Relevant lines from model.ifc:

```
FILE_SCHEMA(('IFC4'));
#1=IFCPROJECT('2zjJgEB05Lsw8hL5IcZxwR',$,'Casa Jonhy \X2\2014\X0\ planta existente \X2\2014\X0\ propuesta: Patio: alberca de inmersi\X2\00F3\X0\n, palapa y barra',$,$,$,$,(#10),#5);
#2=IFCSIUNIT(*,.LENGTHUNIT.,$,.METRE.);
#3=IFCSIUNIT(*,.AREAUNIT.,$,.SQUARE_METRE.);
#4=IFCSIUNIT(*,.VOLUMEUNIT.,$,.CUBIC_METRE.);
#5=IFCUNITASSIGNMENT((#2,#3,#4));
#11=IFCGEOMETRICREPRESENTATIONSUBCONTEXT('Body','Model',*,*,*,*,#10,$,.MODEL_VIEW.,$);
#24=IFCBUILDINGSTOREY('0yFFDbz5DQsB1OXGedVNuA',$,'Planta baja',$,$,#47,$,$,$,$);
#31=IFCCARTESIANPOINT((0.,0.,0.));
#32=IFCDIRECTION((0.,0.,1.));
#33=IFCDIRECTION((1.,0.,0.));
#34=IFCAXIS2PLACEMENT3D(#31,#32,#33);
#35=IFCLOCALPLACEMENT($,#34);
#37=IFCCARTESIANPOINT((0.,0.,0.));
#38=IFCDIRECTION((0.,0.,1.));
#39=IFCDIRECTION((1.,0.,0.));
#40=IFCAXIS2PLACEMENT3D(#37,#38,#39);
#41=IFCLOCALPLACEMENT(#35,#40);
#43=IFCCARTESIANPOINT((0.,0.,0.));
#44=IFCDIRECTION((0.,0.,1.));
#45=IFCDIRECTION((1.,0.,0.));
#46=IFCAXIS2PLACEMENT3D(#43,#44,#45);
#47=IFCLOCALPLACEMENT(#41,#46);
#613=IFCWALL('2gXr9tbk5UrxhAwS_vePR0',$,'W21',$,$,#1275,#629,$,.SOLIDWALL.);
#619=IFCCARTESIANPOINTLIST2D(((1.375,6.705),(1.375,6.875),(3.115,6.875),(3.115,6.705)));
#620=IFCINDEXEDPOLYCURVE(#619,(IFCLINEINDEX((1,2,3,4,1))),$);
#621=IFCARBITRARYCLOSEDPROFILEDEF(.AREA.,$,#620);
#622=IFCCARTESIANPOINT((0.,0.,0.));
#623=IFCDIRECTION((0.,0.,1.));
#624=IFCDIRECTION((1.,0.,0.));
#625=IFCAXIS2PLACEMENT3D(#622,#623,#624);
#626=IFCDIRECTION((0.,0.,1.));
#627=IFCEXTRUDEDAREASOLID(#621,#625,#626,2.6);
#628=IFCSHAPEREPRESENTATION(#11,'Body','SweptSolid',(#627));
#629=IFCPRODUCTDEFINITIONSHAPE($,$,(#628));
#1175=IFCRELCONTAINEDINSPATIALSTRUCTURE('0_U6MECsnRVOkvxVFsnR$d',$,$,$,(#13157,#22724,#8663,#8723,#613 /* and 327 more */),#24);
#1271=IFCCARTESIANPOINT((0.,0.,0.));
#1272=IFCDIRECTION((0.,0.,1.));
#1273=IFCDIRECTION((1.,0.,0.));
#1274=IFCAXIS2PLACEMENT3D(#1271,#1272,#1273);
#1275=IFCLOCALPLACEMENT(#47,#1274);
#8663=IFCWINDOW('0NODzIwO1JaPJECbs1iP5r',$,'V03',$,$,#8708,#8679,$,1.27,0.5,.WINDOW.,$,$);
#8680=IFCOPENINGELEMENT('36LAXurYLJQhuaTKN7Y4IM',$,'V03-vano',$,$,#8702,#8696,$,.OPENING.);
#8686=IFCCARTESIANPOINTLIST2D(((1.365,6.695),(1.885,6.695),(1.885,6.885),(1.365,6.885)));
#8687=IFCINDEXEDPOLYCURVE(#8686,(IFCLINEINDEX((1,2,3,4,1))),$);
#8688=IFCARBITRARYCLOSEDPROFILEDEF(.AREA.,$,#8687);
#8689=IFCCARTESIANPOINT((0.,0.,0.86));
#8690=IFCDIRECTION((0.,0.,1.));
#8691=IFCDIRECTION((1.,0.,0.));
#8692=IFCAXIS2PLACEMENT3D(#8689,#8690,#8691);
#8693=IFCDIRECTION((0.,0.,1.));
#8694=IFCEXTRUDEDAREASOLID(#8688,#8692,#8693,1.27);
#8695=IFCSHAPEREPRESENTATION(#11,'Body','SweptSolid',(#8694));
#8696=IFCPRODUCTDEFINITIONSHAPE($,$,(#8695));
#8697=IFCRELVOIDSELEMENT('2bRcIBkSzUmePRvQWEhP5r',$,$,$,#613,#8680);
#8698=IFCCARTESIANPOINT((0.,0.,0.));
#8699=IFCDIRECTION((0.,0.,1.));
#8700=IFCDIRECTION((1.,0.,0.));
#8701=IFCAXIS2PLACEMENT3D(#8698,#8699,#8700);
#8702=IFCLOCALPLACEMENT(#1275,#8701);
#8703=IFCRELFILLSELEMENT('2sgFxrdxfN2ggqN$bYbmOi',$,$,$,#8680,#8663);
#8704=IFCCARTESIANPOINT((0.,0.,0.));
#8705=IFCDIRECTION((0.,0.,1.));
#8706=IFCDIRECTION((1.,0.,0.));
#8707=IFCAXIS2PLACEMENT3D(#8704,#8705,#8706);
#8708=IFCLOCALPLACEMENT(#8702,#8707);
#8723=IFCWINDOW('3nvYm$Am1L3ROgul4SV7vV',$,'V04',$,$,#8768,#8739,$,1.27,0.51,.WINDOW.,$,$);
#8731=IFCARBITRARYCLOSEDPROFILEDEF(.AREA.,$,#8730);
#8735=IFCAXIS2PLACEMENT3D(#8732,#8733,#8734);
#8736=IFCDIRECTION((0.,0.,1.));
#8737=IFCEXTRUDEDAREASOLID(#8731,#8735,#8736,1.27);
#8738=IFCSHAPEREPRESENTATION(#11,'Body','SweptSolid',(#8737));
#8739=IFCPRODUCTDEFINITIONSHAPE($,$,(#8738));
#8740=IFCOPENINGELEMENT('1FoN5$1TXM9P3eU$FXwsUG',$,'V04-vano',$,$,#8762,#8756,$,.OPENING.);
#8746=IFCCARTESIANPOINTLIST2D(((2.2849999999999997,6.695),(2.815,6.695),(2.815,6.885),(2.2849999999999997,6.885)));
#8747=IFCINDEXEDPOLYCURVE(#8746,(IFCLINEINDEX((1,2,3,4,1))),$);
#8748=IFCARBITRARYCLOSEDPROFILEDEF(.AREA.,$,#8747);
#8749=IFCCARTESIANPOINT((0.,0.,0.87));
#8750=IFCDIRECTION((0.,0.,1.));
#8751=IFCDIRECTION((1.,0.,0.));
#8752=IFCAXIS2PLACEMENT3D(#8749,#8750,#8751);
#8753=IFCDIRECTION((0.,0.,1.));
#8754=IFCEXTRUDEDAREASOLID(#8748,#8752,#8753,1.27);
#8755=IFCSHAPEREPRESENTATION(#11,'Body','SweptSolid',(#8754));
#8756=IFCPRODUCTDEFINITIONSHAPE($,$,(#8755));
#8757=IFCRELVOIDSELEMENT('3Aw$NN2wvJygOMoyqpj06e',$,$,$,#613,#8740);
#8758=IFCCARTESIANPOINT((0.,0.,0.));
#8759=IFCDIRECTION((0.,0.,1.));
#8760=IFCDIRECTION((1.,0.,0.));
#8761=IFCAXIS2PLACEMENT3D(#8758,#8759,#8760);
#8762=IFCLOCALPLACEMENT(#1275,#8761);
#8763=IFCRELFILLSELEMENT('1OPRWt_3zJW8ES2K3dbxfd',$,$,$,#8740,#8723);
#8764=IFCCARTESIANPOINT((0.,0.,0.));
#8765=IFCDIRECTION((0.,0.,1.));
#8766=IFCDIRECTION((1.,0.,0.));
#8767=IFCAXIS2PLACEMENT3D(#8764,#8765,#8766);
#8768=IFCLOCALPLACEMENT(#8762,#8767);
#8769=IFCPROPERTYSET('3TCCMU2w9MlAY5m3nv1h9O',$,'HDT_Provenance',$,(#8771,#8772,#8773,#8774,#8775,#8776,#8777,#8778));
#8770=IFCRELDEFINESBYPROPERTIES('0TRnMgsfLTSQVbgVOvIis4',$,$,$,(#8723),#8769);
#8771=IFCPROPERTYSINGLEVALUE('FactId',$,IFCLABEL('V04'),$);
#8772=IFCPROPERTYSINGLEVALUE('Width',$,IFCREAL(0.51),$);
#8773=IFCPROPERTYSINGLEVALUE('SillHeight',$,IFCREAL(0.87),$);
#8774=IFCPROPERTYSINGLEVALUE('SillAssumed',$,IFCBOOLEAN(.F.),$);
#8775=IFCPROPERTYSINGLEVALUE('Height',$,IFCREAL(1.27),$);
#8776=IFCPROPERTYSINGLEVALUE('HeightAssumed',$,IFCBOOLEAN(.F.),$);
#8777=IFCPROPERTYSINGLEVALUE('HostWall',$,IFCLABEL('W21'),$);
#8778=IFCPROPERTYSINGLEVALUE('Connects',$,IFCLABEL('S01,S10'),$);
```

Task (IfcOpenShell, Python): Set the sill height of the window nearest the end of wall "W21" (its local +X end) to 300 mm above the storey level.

```python
import numpy as np
import ifcopenshell
import ifcopenshell.api.geometry
import ifcopenshell.api.pset
import ifcopenshell.geom
import ifcopenshell.util.element
import ifcopenshell.util.placement
import ifcopenshell.util.shape
import ifcopenshell.util.unit

model = ifcopenshell.open("model.ifc")
unit_scale = ifcopenshell.util.unit.calculate_unit_scale(model)

window = model.by_id(8723)
opening = window.FillsVoids[0].RelatingOpeningElement
storey = ifcopenshell.util.element.get_container(window, ifc_class="IfcBuildingStorey")
level = ifcopenshell.util.placement.get_local_placement(storey.ObjectPlacement)[2, 3]

# The opening's origin need not be at the sill, so measure its lowest point.
shape = ifcopenshell.geom.create_shape(ifcopenshell.geom.settings(), opening)
bottom = ifcopenshell.util.shape.get_shape_bottom_elevation(shape, shape.geometry) / unit_scale
dz = level + 0.3 / unit_scale - bottom

shift = np.array([0.0, 0.0, dz])
# The window is placed relative to its opening, so it follows when the opening moves.
matrix = ifcopenshell.util.placement.get_local_placement(opening.ObjectPlacement)
matrix[:3, 3] += shift
ifcopenshell.api.geometry.edit_object_placement(
    model, product=opening, matrix=matrix, is_si=False, should_transform_children=True
)

# Keep the stored heights in step.
pset = model.by_id(ifcopenshell.util.element.get_pset(window, "HDT_Provenance", should_inherit=False)["id"])
ifcopenshell.api.pset.edit_pset(model, pset=pset, properties={
    "SillHeight": model.create_entity("IfcReal", ifcopenshell.util.element.get_pset(window, "HDT_Provenance", "SillHeight") + dz),
})

print(f"moved by {dz * unit_scale:+.3f} m")

model.write("model_updated.ifc")
```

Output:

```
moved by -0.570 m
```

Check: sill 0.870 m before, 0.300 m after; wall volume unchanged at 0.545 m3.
